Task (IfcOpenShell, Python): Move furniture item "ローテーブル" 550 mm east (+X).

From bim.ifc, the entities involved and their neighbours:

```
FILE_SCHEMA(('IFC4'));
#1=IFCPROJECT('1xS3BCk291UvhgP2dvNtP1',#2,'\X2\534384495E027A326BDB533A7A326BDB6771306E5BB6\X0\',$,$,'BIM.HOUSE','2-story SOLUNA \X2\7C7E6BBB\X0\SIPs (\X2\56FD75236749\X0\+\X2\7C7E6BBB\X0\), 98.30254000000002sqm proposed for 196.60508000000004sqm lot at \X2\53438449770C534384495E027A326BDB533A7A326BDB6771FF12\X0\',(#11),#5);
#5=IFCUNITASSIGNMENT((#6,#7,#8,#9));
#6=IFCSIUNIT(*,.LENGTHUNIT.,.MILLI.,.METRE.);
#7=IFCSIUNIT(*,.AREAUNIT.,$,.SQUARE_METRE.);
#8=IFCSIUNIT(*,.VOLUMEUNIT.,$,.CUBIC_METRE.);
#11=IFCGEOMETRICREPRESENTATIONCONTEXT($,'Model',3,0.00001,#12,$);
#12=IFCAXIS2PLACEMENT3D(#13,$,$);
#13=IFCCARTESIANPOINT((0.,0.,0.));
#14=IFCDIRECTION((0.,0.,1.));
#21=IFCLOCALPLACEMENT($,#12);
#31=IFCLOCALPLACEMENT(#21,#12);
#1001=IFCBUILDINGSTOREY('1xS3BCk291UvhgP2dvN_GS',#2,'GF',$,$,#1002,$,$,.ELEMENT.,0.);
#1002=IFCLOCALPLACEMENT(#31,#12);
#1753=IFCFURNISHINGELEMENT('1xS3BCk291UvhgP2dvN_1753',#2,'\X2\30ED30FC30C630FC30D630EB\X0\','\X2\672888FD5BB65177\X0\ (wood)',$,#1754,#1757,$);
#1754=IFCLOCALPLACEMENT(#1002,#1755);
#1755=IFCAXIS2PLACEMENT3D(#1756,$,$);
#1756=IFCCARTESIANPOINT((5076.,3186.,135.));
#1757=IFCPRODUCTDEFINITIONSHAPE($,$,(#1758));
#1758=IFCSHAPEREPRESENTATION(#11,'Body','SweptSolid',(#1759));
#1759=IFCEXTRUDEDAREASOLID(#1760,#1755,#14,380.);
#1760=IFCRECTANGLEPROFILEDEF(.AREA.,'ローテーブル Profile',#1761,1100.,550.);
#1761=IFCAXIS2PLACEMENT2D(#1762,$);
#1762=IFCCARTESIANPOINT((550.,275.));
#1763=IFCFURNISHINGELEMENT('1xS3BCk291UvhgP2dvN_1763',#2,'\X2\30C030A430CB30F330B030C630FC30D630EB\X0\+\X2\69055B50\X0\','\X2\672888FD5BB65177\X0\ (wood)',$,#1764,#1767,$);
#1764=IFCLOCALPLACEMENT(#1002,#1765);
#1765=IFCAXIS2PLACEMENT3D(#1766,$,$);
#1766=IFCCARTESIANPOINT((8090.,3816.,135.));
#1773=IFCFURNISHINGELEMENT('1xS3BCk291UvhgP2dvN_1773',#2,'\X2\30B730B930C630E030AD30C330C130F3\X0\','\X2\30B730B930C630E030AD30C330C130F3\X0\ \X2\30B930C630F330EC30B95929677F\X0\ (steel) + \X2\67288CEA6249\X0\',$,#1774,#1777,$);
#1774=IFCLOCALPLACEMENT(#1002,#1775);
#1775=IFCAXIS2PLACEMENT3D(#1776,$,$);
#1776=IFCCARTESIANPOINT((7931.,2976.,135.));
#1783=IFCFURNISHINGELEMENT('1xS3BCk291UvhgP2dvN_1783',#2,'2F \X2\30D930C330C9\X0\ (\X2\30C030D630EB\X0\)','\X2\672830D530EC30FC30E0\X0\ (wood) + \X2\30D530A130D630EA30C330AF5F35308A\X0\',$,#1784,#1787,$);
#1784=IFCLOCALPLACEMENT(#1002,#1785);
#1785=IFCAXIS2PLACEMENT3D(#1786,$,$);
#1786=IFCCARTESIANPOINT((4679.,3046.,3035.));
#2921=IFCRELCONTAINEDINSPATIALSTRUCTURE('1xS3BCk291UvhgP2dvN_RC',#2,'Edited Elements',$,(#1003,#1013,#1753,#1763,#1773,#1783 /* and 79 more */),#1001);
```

```python
import ifcopenshell
import ifcopenshell.api.geometry
import ifcopenshell.util.placement
import ifcopenshell.util.unit

model = ifcopenshell.open("bim.ifc")
unit_scale = ifcopenshell.util.unit.calculate_unit_scale(model)

item = model.by_guid("1xS3BCk291UvhgP2dvN_1753")
matrix = ifcopenshell.util.placement.get_local_placement(item.ObjectPlacement)
matrix[0, 3] += 0.55 / unit_scale
ifcopenshell.api.geometry.edit_object_placement(model, product=item, matrix=matrix, is_si=False)

print(ifcopenshell.util.placement.get_local_placement(item.ObjectPlacement).round(3) + 0.0)

model.write("bim_rev.ifc")
```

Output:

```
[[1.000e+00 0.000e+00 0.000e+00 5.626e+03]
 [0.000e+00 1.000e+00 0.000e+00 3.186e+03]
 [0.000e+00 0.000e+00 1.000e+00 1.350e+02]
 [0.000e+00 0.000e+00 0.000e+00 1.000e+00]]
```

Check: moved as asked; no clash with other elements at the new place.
